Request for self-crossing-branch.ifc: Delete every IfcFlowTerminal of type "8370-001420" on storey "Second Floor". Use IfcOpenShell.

First a look at what the model holds.

```python
import ifcopenshell
import ifcopenshell.util.element

model = ifcopenshell.open("self-crossing-branch.ifc")
print(model.schema)
storey = next(s for s in model.by_type("IfcBuildingStorey") if s.Name == "Second Floor")
terminals = [e for e in ifcopenshell.util.element.get_decomposition(storey) if e.is_a("IfcFlowTerminal")]
seen = {}
for e in terminals:
    element_type = ifcopenshell.util.element.get_type(e)
    name = element_type.Name if element_type not in (None, e) else None
    seen[name] = seen.get(name, 0) + 1
for name, count in sorted(seen.items(), key=str):
    print(count, "x", name)
```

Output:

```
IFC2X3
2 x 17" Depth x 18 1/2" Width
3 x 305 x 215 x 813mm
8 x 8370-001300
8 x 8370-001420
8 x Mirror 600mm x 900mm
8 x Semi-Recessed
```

```python
import ifcopenshell
import ifcopenshell.api.root
import ifcopenshell.util.element

model = ifcopenshell.open("self-crossing-branch.ifc")

storey = next(s for s in model.by_type("IfcBuildingStorey") if s.Name == "Second Floor")
terminals = [e for e in ifcopenshell.util.element.get_decomposition(storey) if e.is_a("IfcFlowTerminal")]
targets = [e for e in terminals if (t := ifcopenshell.util.element.get_type(e)) not in (None, e) and t.Name == "8370-001420"]

for e in targets:
    ifcopenshell.api.root.remove_product(model, product=e)
print(len(targets), "removed")

model.write("self-crossing-branch_updated.ifc")
```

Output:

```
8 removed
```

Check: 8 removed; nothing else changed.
